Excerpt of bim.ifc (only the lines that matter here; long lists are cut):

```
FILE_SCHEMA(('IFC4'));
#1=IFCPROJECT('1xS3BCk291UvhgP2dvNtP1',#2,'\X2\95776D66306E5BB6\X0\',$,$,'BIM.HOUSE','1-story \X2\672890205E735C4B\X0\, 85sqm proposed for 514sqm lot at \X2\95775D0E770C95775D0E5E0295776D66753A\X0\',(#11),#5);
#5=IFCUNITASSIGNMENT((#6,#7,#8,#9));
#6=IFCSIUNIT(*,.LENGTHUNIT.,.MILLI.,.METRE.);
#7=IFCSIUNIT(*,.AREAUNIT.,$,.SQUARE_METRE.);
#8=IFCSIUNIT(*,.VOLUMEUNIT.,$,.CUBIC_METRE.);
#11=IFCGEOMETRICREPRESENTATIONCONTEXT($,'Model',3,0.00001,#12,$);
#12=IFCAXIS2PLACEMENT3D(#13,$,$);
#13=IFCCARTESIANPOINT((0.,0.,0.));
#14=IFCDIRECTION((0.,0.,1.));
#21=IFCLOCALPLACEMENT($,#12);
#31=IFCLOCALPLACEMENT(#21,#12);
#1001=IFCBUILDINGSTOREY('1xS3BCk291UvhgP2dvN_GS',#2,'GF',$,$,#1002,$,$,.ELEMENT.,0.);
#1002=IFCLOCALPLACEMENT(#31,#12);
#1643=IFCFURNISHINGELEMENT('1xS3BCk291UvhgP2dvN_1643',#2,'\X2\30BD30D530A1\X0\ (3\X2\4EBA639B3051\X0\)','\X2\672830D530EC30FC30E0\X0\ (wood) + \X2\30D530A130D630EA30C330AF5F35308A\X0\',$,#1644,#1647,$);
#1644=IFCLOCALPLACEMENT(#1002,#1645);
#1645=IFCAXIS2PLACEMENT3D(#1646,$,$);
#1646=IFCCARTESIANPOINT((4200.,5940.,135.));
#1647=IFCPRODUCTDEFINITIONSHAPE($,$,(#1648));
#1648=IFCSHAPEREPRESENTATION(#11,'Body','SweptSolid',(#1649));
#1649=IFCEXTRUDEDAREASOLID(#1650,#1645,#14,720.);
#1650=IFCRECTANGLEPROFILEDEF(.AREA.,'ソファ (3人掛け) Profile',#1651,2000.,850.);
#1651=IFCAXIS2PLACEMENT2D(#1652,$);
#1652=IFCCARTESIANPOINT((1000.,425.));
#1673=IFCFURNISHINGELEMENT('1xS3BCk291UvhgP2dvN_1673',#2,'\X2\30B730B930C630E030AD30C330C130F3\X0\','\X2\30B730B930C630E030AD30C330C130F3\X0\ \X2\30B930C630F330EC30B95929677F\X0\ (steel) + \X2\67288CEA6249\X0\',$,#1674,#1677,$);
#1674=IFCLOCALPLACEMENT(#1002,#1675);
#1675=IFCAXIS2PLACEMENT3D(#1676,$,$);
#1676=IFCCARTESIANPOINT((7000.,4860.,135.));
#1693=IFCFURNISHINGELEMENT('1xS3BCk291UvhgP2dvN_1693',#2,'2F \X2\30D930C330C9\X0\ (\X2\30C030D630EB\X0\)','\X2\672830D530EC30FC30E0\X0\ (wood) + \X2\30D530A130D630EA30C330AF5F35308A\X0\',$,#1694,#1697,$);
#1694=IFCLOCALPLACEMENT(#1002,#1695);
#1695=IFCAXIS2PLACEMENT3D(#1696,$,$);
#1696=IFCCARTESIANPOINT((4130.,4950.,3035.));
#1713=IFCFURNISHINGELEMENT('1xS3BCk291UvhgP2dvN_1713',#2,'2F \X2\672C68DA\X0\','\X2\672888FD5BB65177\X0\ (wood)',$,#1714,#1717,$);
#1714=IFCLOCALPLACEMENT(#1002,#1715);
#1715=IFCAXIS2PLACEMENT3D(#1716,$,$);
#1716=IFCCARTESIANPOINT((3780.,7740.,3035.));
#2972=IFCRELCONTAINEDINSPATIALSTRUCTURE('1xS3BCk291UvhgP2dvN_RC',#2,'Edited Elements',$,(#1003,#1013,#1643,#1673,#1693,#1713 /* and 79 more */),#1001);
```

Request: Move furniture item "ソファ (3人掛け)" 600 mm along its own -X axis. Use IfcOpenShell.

```python
import ifcopenshell
import ifcopenshell.api.geometry
import ifcopenshell.util.placement

model = ifcopenshell.open("bim.ifc")

item = model.by_id(1643)
matrix = ifcopenshell.util.placement.get_local_placement(item.ObjectPlacement)
matrix[:3, 3] -= matrix[:3, 0] * 600.0
ifcopenshell.api.geometry.edit_object_placement(model, product=item, matrix=matrix, is_si=False)

print(ifcopenshell.util.placement.get_local_placement(item.ObjectPlacement).round(3) + 0.0)

model.write("bim-out.ifc")
```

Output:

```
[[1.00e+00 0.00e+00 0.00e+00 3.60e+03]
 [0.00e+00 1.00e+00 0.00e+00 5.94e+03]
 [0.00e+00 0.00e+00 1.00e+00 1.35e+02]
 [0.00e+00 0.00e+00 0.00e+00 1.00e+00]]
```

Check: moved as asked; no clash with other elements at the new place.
